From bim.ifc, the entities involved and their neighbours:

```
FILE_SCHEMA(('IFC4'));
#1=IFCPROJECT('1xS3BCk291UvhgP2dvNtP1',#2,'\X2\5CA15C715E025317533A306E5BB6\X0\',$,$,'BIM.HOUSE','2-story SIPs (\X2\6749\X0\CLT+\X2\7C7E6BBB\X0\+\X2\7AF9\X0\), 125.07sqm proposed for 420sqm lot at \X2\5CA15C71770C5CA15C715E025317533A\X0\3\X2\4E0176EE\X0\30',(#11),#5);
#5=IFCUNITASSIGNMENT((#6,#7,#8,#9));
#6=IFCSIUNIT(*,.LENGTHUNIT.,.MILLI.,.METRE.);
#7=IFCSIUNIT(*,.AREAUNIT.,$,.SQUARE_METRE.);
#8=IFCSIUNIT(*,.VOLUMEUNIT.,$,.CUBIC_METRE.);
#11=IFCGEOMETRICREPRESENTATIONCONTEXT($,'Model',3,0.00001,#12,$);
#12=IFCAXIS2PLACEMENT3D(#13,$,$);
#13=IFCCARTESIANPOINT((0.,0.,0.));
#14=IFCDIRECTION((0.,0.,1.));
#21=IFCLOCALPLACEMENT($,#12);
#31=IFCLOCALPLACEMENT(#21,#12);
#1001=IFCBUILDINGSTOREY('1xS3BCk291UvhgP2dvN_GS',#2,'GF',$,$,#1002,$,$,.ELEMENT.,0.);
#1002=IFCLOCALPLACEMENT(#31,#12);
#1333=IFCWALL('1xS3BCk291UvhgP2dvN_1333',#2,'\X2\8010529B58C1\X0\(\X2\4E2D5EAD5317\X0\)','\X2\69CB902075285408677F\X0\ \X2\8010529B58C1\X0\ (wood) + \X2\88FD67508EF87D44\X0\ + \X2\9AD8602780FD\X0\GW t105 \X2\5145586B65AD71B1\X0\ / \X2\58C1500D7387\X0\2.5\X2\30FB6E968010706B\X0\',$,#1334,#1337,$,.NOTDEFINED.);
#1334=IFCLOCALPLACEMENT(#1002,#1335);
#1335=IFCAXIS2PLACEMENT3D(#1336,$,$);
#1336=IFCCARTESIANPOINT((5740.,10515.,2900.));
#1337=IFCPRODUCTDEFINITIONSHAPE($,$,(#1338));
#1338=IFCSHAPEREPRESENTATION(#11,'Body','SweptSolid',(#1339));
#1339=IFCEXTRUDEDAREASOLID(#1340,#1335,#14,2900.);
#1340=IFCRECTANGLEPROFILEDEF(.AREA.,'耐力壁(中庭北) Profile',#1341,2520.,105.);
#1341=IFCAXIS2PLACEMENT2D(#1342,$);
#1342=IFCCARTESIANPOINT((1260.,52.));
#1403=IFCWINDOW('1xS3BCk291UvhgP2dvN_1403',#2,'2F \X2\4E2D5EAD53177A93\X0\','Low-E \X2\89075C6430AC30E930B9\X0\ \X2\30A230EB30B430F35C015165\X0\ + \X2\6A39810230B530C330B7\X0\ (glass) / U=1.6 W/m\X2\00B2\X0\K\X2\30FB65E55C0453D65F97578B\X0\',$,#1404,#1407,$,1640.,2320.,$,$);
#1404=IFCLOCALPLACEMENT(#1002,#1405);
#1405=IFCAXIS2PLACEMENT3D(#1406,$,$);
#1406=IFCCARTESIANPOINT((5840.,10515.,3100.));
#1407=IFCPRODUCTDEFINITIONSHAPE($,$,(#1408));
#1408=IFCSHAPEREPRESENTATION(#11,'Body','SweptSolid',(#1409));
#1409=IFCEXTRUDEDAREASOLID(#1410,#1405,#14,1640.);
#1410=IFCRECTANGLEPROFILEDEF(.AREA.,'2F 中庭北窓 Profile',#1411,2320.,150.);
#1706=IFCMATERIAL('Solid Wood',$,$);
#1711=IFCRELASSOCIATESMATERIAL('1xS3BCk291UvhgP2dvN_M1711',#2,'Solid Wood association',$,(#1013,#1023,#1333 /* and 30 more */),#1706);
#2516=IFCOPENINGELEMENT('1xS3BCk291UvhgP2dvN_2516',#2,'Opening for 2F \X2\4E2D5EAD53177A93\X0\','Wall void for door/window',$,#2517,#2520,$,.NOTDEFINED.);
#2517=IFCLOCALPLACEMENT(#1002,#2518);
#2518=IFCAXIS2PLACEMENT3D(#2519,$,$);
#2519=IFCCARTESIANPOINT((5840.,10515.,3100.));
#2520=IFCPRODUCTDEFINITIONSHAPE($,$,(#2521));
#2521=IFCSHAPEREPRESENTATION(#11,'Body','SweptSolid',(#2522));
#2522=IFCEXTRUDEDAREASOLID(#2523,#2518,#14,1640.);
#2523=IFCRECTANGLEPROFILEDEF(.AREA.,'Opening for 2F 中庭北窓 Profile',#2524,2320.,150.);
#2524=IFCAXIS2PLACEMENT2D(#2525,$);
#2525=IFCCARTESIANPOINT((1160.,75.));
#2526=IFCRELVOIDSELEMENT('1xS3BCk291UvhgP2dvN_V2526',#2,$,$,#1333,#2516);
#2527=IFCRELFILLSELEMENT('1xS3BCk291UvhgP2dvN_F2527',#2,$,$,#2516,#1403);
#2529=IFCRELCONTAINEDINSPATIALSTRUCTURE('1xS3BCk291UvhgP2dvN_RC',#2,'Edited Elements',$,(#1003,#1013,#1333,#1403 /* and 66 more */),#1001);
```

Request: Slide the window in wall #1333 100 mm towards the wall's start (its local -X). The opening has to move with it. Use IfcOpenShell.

```python
import ifcopenshell
import ifcopenshell.api.geometry
import ifcopenshell.util.placement

model = ifcopenshell.open("bim.ifc")

window = model.by_guid("1xS3BCk291UvhgP2dvN_1403")
opening = window.FillsVoids[0].RelatingOpeningElement
wall = opening.VoidsElements[0].RelatingBuildingElement

wall_matrix = ifcopenshell.util.placement.get_local_placement(wall.ObjectPlacement)
shift = wall_matrix[:3, 0] * -100.0
before = ifcopenshell.util.placement.get_local_placement(window.ObjectPlacement)[:3, 3].copy()

# The window is not placed relative to its opening, so move both.
for product in (opening, window):
    matrix = ifcopenshell.util.placement.get_local_placement(product.ObjectPlacement)
    matrix[:3, 3] += shift
    ifcopenshell.api.geometry.edit_object_placement(model, product=product, matrix=matrix, is_si=False)

after = ifcopenshell.util.placement.get_local_placement(window.ObjectPlacement)[:3, 3]
print("window moved by", (after - before).round(3) + 0.0)

model.write("bim-out.ifc")
```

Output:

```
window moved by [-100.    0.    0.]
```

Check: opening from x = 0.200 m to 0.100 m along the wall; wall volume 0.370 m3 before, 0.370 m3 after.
